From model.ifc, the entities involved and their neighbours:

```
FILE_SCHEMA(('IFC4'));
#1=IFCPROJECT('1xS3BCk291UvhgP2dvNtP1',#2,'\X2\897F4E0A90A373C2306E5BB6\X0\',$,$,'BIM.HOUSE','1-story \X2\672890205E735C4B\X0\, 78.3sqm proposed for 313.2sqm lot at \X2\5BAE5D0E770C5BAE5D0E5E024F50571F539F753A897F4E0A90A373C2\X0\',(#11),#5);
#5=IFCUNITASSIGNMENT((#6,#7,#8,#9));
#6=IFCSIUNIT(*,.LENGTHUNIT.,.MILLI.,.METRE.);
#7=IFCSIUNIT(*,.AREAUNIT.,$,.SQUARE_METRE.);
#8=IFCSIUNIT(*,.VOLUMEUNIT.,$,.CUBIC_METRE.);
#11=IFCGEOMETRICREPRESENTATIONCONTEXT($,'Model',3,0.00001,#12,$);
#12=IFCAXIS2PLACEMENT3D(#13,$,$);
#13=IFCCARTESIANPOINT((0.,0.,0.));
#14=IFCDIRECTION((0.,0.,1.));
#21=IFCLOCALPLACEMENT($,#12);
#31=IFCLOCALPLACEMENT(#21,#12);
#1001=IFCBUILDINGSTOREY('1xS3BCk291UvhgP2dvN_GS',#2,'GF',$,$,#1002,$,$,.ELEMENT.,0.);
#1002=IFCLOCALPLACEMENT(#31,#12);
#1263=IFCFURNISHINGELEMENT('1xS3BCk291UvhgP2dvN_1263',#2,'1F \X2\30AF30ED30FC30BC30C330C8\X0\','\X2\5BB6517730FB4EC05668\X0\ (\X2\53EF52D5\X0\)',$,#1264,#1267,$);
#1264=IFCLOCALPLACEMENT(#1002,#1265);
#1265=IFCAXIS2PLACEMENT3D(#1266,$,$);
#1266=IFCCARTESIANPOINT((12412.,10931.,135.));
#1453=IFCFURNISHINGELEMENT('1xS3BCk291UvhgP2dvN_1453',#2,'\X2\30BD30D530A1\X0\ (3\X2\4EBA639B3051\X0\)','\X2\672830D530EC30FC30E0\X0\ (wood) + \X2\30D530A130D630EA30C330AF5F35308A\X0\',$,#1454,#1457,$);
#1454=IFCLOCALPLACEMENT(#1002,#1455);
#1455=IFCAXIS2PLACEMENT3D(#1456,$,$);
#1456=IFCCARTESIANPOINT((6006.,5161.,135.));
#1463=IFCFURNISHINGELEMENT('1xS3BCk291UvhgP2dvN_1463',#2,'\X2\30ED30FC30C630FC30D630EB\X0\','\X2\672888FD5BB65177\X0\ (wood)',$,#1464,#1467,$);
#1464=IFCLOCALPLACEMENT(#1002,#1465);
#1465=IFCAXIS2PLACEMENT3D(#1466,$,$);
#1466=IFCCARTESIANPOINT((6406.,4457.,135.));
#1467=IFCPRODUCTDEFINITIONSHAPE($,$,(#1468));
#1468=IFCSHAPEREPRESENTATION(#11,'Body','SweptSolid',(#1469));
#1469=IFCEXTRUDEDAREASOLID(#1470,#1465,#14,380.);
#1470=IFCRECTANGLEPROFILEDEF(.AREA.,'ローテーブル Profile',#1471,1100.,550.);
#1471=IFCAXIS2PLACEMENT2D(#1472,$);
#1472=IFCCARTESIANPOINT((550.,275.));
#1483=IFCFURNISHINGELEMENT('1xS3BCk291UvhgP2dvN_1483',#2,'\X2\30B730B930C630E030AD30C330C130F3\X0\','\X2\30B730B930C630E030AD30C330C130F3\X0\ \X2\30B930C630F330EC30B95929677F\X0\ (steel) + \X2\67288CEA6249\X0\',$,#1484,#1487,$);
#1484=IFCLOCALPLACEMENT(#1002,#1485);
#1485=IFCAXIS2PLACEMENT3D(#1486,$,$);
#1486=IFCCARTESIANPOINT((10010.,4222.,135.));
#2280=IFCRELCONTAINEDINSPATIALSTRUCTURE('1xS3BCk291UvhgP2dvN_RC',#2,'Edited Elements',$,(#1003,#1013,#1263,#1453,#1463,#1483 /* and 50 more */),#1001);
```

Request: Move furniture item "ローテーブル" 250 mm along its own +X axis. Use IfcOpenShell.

```python
import ifcopenshell
import ifcopenshell.api.geometry
import ifcopenshell.util.placement
import ifcopenshell.util.unit

model = ifcopenshell.open("model.ifc")
unit_scale = ifcopenshell.util.unit.calculate_unit_scale(model)

item = model.by_guid("1xS3BCk291UvhgP2dvN_1463")
matrix = ifcopenshell.util.placement.get_local_placement(item.ObjectPlacement)
matrix[:3, 3] += matrix[:3, 0] * 0.25 / unit_scale
ifcopenshell.api.geometry.edit_object_placement(model, product=item, matrix=matrix, is_si=False)

print(ifcopenshell.util.placement.get_local_placement(item.ObjectPlacement).round(3) + 0.0)

model.write("model-out.ifc")
```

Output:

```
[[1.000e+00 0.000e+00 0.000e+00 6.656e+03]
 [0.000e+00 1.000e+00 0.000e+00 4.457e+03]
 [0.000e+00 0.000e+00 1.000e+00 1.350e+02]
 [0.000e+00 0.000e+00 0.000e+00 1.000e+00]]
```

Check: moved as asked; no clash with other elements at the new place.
